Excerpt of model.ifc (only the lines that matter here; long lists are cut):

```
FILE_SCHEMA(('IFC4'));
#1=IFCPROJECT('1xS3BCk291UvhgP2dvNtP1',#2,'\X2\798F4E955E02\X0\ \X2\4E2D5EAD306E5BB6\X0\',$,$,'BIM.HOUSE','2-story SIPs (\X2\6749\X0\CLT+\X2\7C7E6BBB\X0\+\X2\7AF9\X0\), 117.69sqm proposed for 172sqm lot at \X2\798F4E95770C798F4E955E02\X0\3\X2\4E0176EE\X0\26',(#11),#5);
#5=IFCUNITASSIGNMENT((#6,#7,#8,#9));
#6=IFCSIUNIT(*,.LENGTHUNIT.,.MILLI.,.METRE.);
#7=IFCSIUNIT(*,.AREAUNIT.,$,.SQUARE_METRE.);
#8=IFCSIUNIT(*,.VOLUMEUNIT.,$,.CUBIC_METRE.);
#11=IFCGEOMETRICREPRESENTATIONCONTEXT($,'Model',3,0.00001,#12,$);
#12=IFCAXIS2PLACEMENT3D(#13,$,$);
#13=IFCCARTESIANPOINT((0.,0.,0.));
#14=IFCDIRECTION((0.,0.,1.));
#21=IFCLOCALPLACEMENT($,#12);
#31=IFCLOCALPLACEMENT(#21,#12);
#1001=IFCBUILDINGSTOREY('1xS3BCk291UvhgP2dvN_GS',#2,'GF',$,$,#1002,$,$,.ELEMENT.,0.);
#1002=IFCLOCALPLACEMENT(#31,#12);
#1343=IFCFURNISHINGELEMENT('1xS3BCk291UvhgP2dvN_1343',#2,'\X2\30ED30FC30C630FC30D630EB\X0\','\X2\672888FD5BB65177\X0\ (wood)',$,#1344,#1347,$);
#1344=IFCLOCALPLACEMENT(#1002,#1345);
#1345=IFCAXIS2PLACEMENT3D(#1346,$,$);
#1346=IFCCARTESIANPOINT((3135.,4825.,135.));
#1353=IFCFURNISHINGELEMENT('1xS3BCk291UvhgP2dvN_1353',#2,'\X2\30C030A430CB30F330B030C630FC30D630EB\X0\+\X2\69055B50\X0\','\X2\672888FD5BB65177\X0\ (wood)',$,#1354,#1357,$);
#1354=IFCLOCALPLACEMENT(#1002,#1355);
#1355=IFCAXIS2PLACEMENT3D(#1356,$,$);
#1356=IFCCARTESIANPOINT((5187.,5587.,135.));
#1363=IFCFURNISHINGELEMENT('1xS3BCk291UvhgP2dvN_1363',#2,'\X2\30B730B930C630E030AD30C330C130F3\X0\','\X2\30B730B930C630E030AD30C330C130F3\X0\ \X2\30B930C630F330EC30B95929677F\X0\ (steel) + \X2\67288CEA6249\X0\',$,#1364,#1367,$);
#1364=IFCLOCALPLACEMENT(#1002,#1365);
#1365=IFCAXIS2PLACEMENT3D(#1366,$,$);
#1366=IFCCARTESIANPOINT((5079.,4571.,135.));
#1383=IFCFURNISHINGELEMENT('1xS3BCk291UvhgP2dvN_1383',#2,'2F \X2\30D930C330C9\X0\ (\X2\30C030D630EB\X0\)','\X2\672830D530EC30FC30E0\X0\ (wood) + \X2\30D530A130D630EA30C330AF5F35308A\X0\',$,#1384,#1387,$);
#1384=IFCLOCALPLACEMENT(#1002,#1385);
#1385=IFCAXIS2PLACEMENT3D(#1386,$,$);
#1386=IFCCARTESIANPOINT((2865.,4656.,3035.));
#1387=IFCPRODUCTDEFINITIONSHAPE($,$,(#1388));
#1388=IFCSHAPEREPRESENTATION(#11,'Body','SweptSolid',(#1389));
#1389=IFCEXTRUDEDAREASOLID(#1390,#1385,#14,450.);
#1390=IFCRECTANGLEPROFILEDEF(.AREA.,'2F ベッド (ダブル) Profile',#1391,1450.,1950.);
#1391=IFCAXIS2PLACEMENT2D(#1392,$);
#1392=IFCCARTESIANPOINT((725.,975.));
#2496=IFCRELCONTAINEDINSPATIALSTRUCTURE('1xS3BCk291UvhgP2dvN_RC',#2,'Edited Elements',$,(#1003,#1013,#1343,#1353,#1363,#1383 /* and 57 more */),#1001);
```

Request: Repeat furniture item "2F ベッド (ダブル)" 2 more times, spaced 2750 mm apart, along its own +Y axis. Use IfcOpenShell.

```python
import ifcopenshell
import ifcopenshell.api.geometry
import ifcopenshell.api.root
import ifcopenshell.util.element
import ifcopenshell.util.placement
import ifcopenshell.util.unit

model = ifcopenshell.open("model.ifc")
unit_scale = ifcopenshell.util.unit.calculate_unit_scale(model)


def reuse_history(source, copy):
    """copy_class also copies each property set's owner history, people and application; keep the originals."""
    for rel in copy.IsDefinedBy:
        if rel.is_a("IfcRelDefinesByProperties") and (history := rel.RelatingPropertyDefinition.OwnerHistory):
            rel.RelatingPropertyDefinition.OwnerHistory = source.OwnerHistory
            ifcopenshell.util.element.remove_deep2(model, history)


source = model.by_id(1383)
base = ifcopenshell.util.placement.get_local_placement(source.ObjectPlacement)
step = base[:3, 1] * 2.75 / unit_scale

for i in range(1, 3):
    copy = ifcopenshell.api.root.copy_class(model, product=source)
    copy.Representation = ifcopenshell.util.element.copy_deep(
        model, source.Representation, exclude=["IfcGeometricRepresentationContext", "IfcRepresentationMap"]
    )
    reuse_history(source, copy)
    matrix = base.copy()
    matrix[:3, 3] += i * step
    print("added at", matrix[:3, 3].round(3) + 0.0)
    ifcopenshell.api.geometry.edit_object_placement(model, product=copy, matrix=matrix, is_si=False)

model.write("model_rev.ifc")
```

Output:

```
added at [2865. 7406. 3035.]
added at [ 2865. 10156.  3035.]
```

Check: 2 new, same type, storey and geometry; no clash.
